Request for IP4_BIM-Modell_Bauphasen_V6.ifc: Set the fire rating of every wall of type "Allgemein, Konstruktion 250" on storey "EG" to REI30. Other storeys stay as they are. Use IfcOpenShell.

First a look at what the model holds.

```python
import ifcopenshell
import ifcopenshell.util.element

model = ifcopenshell.open("IP4_BIM-Modell_Bauphasen_V6.ifc")
print(model.schema)
storey = next(s for s in model.by_type("IfcBuildingStorey") if s.Name == "EG")
walls = [e for e in ifcopenshell.util.element.get_decomposition(storey) if e.is_a("IfcWall")]
seen = {}
for e in walls:
    element_type = ifcopenshell.util.element.get_type(e)
    key = (element_type.Name if element_type != e and element_type else None, ifcopenshell.util.element.get_pset(e, "Pset_WallCommon", "FireRating"))
    seen[key] = seen.get(key, 0) + 1
for (name, value), count in sorted(seen.items(), key=str):
    print(count, "x", name, "|", value)
```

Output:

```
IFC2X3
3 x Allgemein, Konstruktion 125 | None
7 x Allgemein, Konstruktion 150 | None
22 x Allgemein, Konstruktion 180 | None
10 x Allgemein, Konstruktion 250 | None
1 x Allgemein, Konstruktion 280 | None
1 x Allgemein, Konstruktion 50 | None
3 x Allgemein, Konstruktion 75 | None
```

```python
import ifcopenshell
import ifcopenshell.api.pset
import ifcopenshell.util.element

model = ifcopenshell.open("IP4_BIM-Modell_Bauphasen_V6.ifc")

storey = next(s for s in model.by_type("IfcBuildingStorey") if s.Name == "EG")
walls = [e for e in ifcopenshell.util.element.get_decomposition(storey) if e.is_a("IfcWall")]

count = 0
for e in walls:
    element_type = ifcopenshell.util.element.get_type(e)
    if element_type in (None, e) or element_type.Name != "Allgemein, Konstruktion 250":
        continue
    # add_pset returns the element's existing set when there is one.
    pset = ifcopenshell.api.pset.add_pset(model, product=e, name="Pset_WallCommon")
    ifcopenshell.api.pset.edit_pset(model, pset=pset, properties={"FireRating": "REI30"})
    count += 1

print(count, "walls updated")

model.write("IP4_BIM-Modell_Bauphasen_V6_v2.ifc")
```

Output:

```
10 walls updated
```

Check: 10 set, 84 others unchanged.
